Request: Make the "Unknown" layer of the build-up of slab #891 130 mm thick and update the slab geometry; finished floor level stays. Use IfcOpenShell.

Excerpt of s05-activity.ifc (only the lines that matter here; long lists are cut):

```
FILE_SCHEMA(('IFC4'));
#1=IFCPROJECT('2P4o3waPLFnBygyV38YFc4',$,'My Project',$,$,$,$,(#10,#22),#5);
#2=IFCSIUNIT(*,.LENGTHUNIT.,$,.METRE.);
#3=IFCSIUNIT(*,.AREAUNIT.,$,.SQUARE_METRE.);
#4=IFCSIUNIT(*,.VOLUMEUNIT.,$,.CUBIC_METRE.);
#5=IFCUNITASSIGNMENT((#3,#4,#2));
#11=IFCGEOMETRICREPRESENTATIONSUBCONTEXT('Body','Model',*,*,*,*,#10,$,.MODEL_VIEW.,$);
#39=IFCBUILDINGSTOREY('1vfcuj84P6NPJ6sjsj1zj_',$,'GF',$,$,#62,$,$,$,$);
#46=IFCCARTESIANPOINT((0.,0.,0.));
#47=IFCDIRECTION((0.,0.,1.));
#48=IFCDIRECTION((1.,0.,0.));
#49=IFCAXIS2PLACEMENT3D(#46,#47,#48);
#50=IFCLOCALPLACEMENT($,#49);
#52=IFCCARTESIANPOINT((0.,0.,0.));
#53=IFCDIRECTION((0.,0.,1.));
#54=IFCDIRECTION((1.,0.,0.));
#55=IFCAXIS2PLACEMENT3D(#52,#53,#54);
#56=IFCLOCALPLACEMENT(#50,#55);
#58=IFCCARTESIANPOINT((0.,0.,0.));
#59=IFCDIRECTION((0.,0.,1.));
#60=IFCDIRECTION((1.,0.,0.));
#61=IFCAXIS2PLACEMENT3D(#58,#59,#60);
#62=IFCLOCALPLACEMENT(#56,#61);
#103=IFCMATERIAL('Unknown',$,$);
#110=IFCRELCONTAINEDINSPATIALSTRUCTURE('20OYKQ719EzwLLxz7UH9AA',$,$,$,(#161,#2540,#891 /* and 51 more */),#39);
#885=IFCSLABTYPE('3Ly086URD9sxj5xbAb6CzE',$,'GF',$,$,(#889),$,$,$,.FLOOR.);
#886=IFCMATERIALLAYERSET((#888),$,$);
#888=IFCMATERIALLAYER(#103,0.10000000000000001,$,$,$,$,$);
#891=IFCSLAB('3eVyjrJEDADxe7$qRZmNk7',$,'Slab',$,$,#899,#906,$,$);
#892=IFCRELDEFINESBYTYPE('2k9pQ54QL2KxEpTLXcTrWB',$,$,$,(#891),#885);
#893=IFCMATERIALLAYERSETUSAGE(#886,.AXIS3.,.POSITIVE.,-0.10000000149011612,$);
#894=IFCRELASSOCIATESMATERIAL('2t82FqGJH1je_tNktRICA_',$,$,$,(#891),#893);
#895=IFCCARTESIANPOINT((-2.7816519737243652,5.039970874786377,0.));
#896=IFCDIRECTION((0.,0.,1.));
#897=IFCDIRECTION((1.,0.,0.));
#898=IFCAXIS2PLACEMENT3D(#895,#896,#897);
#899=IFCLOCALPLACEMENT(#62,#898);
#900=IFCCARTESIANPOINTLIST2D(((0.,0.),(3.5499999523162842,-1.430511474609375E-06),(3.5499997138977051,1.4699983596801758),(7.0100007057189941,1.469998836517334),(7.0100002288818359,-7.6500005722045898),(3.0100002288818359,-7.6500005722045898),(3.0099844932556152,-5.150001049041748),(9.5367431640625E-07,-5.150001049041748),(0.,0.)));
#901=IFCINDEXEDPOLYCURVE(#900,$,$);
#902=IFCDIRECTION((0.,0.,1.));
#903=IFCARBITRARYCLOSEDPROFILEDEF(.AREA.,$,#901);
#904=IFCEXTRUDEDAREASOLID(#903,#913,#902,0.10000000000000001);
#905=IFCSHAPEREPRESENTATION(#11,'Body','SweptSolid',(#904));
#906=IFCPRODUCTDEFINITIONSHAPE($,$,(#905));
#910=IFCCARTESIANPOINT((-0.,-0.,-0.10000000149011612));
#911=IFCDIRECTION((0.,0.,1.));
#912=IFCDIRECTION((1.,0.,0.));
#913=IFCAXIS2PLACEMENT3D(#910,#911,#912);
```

```python
import ifcopenshell
import ifcopenshell.util.element
import ifcopenshell.util.representation

model = ifcopenshell.open("s05-activity.ifc")

layer_set = model.by_id(886)
layer = next(l for l in layer_set.MaterialLayers if l.Material and l.Material.Name == "Unknown")
change = 0.13 - layer.LayerThickness
layer.LayerThickness += change

# Geometry does not follow the layer set by itself.
slabs = [e for e in ifcopenshell.util.element.get_elements_by_material(model, layer_set) if e.is_a("IfcSlab")]
for slab in sorted(slabs, key=lambda e: e.id()):
    body = ifcopenshell.util.representation.get_representation(slab, "Model", "Body")
    solid = body.Items[0]
    old_depth = solid.Depth
    solid.Depth += change
    # Extruded upwards: lower the start of the extrusion so the top stays.
    x, y, z = solid.Position.Location.Coordinates
    solid.Position.Location = model.createIfcCartesianPoint((x, y, z - change))
    print(slab.id(), f"{old_depth:g} -> {solid.Depth:g}")

# The layers are counted up from the underside, which has moved.
for usage in {ifcopenshell.util.element.get_material(slab) for slab in slabs}:
    usage.OffsetFromReferenceLine -= change

model.write("s05-activity_rev.ifc")
```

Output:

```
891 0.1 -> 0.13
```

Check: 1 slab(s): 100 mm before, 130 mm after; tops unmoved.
